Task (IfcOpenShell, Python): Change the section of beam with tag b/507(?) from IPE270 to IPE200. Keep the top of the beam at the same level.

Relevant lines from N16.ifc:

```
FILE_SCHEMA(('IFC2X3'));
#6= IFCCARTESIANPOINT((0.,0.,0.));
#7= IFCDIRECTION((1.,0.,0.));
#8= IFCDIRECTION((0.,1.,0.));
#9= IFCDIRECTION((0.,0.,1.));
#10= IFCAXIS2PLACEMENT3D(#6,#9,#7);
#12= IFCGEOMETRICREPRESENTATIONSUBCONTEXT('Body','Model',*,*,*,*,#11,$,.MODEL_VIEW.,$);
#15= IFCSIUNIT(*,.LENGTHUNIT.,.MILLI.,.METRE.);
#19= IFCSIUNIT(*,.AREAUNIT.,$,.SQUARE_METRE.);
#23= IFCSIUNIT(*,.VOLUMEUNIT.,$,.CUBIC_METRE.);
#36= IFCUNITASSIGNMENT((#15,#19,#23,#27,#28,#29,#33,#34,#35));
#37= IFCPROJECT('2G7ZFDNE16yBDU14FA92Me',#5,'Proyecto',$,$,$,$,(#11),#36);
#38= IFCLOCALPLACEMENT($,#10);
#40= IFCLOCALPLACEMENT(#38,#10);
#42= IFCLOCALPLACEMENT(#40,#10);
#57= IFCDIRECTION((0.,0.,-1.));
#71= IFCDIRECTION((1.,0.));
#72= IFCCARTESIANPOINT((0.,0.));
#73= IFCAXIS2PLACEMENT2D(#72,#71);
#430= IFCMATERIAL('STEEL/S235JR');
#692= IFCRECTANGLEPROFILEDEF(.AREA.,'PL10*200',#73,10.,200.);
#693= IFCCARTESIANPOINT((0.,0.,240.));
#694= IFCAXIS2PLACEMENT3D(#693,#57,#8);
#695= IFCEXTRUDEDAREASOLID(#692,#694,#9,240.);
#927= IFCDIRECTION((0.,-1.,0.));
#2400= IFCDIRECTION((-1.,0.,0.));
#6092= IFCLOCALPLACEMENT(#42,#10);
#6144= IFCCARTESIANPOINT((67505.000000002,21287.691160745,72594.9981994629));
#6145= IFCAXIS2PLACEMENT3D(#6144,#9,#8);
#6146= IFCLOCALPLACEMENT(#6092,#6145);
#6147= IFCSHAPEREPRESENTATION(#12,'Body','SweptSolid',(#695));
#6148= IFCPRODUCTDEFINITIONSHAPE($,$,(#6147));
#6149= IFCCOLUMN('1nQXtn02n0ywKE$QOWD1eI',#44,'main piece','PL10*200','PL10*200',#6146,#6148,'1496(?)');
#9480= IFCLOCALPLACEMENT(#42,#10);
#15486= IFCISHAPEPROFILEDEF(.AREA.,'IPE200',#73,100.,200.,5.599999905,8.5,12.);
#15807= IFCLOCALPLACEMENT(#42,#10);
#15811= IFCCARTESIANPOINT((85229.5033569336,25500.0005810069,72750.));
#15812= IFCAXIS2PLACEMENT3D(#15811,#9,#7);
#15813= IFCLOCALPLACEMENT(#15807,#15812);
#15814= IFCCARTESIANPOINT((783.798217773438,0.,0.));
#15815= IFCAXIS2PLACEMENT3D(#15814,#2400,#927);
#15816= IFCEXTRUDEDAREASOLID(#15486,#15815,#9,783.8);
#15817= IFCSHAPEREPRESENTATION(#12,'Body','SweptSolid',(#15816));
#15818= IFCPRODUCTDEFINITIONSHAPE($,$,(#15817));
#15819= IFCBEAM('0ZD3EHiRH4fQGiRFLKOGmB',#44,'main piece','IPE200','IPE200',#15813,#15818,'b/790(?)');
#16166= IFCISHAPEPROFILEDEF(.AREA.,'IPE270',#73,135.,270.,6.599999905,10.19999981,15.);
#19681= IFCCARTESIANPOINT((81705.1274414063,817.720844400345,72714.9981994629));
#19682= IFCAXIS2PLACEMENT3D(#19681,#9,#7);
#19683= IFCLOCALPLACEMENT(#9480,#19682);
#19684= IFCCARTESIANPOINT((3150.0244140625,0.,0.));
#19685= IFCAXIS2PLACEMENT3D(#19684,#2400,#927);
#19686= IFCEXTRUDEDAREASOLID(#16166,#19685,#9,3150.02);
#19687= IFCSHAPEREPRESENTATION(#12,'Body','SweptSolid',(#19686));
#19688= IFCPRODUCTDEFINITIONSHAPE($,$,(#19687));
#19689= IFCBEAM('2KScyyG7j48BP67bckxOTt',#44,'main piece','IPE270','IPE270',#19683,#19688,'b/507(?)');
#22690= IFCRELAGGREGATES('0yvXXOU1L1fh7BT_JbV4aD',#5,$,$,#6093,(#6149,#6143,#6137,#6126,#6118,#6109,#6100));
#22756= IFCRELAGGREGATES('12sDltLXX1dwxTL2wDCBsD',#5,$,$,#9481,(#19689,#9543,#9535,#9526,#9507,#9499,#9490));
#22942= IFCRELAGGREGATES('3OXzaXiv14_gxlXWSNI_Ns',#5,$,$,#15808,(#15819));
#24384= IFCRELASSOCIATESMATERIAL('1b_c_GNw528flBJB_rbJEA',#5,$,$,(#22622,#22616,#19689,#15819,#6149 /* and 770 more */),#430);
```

```python
import ifcopenshell
import ifcopenshell.util.element
import ifcopenshell.util.representation

model = ifcopenshell.open("N16.ifc")

member = model.by_guid("2KScyyG7j48BP67bckxOTt")
source = next(p for p in model.by_type("IfcIShapeProfileDef") if p.ProfileName == "IPE200")

body = ifcopenshell.util.representation.get_representation(member, "Model", "Body")
solid = body.Items[0]
old_profile = solid.SweptArea

# Copy the section's sizes but keep this member's own profile position.
profile = ifcopenshell.util.element.copy(model, source)
# Profiles are centred, so shift by half the change in depth to hold the top.
shift = (old_profile.OverallDepth - profile.OverallDepth) / 2
x, y = old_profile.Position.Location.Coordinates
up = (0.0, 1.0)  # upwards, in the solid's own plane
location = model.createIfcCartesianPoint((x + up[0] * shift, y + up[1] * shift))
profile.Position = model.createIfcAxis2Placement2D(location, old_profile.Position.RefDirection)
solid.SweptArea = profile
if not model.get_total_inverses(old_profile):
    ifcopenshell.util.element.remove_deep2(model, old_profile)
member.Description = member.Description.replace("IPE270", "IPE200")
member.ObjectType = member.ObjectType.replace("IPE270", "IPE200")

print(solid.SweptArea)

model.write("N16-out.ifc")
```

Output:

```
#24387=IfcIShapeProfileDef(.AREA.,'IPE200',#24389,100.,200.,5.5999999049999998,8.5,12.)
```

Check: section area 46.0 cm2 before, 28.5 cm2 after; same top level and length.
